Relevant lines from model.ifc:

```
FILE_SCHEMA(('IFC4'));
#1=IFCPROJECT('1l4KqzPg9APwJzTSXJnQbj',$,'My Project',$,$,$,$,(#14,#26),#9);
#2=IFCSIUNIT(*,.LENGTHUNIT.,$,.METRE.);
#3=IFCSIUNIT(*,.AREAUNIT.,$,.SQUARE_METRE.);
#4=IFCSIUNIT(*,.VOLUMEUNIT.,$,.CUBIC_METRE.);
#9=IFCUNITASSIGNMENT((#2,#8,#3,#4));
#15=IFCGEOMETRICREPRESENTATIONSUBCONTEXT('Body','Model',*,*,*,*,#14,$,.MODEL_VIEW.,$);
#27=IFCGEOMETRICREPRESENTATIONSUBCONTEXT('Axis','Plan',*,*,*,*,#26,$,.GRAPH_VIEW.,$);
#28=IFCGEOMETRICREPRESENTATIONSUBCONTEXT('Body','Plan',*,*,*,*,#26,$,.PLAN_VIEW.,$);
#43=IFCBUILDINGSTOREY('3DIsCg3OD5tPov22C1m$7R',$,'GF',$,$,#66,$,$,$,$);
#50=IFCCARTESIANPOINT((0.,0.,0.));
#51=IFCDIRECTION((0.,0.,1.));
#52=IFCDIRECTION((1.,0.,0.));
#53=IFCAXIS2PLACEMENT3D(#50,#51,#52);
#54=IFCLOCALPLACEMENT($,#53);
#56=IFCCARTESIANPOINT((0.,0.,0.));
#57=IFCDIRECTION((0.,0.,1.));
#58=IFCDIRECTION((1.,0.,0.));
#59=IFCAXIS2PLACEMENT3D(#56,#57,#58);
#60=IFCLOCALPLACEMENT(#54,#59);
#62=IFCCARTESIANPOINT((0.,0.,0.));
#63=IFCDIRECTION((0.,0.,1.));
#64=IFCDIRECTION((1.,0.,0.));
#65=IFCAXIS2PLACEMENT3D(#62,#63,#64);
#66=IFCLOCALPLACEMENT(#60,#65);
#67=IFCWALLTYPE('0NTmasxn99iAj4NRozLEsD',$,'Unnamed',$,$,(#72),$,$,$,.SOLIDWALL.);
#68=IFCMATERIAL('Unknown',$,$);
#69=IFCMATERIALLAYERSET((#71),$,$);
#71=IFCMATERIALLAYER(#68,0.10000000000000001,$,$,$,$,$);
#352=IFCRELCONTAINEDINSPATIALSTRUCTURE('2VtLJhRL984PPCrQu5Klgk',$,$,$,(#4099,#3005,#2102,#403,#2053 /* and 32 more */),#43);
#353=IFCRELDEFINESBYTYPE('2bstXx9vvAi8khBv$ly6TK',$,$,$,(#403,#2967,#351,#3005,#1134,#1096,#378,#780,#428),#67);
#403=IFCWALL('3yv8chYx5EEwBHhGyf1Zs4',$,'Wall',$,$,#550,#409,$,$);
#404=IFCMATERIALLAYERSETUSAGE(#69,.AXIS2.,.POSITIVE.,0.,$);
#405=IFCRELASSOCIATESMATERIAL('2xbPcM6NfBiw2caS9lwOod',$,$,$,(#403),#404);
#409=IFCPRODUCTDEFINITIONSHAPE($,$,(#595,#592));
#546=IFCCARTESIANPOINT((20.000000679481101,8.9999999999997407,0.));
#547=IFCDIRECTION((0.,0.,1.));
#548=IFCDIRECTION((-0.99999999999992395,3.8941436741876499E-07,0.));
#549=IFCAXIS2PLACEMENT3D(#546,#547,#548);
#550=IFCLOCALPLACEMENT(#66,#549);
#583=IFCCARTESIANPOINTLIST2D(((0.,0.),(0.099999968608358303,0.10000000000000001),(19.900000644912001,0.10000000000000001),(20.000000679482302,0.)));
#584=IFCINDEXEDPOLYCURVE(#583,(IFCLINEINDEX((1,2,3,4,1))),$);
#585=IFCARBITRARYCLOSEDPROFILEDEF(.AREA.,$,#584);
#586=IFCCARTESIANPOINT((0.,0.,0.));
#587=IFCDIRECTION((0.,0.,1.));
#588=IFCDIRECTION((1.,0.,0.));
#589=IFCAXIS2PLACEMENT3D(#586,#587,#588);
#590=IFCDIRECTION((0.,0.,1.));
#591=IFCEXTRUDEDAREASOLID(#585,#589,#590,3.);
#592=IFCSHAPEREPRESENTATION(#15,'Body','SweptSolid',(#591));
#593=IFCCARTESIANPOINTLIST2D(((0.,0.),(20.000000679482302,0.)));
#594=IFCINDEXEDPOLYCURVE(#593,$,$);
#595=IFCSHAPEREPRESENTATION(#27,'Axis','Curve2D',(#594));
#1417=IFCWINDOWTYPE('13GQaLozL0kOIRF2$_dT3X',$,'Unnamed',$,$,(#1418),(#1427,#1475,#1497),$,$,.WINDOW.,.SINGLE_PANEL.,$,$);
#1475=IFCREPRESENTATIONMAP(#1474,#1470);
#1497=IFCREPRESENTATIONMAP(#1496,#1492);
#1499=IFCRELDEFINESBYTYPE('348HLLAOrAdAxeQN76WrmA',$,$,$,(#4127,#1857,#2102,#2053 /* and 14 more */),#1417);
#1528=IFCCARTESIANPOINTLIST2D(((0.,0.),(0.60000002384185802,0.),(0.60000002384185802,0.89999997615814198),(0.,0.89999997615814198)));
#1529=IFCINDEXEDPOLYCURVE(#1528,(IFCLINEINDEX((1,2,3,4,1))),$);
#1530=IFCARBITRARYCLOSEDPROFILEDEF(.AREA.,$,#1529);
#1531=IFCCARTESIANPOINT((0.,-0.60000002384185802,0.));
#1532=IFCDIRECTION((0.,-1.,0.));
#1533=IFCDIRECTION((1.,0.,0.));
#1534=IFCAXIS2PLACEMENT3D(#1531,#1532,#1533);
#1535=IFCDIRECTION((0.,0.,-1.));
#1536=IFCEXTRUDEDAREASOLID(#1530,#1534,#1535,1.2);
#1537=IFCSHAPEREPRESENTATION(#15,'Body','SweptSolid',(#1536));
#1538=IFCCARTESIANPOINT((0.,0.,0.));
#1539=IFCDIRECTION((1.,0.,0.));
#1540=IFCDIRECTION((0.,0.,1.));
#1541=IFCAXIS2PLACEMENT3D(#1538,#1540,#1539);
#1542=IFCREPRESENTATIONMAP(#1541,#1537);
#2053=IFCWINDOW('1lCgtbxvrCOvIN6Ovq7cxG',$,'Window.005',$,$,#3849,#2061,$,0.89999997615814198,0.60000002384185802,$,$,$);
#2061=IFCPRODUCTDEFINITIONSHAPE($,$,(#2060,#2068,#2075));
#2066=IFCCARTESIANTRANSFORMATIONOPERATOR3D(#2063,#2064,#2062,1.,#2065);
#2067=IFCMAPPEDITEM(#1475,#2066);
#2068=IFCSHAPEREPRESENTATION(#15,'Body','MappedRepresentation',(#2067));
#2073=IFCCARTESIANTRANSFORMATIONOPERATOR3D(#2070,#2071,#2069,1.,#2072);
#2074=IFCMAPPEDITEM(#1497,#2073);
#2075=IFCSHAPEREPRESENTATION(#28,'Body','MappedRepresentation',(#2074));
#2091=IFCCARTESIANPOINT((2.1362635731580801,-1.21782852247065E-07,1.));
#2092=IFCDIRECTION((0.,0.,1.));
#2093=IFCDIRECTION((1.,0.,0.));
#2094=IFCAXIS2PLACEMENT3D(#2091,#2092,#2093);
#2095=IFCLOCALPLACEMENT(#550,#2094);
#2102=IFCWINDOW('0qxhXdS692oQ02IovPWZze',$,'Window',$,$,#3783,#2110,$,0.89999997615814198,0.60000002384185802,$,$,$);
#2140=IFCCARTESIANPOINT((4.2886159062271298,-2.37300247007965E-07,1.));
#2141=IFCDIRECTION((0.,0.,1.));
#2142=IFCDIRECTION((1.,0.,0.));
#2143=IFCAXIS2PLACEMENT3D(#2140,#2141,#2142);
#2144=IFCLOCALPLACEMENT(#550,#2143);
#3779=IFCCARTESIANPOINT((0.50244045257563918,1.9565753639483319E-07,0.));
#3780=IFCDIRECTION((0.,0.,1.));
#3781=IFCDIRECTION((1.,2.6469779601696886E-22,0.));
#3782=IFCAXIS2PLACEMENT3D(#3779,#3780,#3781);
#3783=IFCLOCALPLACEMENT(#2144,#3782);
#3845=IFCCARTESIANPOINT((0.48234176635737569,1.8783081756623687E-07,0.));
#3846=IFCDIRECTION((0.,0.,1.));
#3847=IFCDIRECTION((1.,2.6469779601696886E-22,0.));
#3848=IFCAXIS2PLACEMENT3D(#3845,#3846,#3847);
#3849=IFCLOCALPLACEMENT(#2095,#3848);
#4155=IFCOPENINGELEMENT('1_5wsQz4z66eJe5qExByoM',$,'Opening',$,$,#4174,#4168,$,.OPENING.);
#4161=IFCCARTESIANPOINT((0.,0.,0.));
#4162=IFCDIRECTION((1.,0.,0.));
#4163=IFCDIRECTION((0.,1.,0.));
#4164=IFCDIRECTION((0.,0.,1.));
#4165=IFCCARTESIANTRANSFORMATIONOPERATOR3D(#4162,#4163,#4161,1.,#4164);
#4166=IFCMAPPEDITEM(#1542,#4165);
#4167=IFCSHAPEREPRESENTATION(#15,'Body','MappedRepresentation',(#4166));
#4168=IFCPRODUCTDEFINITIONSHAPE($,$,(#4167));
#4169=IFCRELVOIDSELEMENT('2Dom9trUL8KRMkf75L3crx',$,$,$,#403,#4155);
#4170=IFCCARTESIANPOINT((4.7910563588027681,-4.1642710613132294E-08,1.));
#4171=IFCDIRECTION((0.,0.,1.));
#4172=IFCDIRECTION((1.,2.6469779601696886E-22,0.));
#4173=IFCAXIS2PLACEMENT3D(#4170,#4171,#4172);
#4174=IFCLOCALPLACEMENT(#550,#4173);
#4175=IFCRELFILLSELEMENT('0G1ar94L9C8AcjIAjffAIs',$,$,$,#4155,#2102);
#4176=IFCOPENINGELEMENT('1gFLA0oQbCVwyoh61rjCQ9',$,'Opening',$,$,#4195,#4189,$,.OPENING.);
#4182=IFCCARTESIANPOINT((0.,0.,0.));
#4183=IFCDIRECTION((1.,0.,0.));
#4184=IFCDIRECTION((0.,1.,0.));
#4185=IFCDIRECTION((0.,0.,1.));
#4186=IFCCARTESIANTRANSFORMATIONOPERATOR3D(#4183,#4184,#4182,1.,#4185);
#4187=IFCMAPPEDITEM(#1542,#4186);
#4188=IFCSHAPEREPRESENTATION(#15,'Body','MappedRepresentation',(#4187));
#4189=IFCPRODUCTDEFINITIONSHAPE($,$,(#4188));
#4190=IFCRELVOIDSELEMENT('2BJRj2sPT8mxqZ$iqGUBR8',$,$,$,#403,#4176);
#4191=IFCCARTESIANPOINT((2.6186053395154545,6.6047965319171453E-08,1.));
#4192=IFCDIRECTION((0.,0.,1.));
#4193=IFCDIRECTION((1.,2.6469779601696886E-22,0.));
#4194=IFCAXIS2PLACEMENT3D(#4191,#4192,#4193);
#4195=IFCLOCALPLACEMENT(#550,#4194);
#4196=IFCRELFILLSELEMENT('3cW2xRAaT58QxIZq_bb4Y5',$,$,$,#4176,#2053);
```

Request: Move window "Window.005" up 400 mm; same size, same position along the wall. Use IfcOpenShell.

```python
import numpy as np
import ifcopenshell
import ifcopenshell.api.geometry
import ifcopenshell.util.placement
import ifcopenshell.util.unit

model = ifcopenshell.open("model.ifc")
unit_scale = ifcopenshell.util.unit.calculate_unit_scale(model)

window = model.by_guid("1lCgtbxvrCOvIN6Ovq7cxG")
opening = window.FillsVoids[0].RelatingOpeningElement
dz = 0.4

shift = np.array([0.0, 0.0, dz])
# The window is not placed relative to its opening, so move both.
for product in (opening, window):
    matrix = ifcopenshell.util.placement.get_local_placement(product.ObjectPlacement)
    matrix[:3, 3] += shift
    ifcopenshell.api.geometry.edit_object_placement(model, product=product, matrix=matrix, is_si=False)

print(f"moved by {dz * unit_scale:+.3f} m")

model.write("model_rev.ifc")
```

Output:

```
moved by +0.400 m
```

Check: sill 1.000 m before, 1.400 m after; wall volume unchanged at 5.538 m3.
